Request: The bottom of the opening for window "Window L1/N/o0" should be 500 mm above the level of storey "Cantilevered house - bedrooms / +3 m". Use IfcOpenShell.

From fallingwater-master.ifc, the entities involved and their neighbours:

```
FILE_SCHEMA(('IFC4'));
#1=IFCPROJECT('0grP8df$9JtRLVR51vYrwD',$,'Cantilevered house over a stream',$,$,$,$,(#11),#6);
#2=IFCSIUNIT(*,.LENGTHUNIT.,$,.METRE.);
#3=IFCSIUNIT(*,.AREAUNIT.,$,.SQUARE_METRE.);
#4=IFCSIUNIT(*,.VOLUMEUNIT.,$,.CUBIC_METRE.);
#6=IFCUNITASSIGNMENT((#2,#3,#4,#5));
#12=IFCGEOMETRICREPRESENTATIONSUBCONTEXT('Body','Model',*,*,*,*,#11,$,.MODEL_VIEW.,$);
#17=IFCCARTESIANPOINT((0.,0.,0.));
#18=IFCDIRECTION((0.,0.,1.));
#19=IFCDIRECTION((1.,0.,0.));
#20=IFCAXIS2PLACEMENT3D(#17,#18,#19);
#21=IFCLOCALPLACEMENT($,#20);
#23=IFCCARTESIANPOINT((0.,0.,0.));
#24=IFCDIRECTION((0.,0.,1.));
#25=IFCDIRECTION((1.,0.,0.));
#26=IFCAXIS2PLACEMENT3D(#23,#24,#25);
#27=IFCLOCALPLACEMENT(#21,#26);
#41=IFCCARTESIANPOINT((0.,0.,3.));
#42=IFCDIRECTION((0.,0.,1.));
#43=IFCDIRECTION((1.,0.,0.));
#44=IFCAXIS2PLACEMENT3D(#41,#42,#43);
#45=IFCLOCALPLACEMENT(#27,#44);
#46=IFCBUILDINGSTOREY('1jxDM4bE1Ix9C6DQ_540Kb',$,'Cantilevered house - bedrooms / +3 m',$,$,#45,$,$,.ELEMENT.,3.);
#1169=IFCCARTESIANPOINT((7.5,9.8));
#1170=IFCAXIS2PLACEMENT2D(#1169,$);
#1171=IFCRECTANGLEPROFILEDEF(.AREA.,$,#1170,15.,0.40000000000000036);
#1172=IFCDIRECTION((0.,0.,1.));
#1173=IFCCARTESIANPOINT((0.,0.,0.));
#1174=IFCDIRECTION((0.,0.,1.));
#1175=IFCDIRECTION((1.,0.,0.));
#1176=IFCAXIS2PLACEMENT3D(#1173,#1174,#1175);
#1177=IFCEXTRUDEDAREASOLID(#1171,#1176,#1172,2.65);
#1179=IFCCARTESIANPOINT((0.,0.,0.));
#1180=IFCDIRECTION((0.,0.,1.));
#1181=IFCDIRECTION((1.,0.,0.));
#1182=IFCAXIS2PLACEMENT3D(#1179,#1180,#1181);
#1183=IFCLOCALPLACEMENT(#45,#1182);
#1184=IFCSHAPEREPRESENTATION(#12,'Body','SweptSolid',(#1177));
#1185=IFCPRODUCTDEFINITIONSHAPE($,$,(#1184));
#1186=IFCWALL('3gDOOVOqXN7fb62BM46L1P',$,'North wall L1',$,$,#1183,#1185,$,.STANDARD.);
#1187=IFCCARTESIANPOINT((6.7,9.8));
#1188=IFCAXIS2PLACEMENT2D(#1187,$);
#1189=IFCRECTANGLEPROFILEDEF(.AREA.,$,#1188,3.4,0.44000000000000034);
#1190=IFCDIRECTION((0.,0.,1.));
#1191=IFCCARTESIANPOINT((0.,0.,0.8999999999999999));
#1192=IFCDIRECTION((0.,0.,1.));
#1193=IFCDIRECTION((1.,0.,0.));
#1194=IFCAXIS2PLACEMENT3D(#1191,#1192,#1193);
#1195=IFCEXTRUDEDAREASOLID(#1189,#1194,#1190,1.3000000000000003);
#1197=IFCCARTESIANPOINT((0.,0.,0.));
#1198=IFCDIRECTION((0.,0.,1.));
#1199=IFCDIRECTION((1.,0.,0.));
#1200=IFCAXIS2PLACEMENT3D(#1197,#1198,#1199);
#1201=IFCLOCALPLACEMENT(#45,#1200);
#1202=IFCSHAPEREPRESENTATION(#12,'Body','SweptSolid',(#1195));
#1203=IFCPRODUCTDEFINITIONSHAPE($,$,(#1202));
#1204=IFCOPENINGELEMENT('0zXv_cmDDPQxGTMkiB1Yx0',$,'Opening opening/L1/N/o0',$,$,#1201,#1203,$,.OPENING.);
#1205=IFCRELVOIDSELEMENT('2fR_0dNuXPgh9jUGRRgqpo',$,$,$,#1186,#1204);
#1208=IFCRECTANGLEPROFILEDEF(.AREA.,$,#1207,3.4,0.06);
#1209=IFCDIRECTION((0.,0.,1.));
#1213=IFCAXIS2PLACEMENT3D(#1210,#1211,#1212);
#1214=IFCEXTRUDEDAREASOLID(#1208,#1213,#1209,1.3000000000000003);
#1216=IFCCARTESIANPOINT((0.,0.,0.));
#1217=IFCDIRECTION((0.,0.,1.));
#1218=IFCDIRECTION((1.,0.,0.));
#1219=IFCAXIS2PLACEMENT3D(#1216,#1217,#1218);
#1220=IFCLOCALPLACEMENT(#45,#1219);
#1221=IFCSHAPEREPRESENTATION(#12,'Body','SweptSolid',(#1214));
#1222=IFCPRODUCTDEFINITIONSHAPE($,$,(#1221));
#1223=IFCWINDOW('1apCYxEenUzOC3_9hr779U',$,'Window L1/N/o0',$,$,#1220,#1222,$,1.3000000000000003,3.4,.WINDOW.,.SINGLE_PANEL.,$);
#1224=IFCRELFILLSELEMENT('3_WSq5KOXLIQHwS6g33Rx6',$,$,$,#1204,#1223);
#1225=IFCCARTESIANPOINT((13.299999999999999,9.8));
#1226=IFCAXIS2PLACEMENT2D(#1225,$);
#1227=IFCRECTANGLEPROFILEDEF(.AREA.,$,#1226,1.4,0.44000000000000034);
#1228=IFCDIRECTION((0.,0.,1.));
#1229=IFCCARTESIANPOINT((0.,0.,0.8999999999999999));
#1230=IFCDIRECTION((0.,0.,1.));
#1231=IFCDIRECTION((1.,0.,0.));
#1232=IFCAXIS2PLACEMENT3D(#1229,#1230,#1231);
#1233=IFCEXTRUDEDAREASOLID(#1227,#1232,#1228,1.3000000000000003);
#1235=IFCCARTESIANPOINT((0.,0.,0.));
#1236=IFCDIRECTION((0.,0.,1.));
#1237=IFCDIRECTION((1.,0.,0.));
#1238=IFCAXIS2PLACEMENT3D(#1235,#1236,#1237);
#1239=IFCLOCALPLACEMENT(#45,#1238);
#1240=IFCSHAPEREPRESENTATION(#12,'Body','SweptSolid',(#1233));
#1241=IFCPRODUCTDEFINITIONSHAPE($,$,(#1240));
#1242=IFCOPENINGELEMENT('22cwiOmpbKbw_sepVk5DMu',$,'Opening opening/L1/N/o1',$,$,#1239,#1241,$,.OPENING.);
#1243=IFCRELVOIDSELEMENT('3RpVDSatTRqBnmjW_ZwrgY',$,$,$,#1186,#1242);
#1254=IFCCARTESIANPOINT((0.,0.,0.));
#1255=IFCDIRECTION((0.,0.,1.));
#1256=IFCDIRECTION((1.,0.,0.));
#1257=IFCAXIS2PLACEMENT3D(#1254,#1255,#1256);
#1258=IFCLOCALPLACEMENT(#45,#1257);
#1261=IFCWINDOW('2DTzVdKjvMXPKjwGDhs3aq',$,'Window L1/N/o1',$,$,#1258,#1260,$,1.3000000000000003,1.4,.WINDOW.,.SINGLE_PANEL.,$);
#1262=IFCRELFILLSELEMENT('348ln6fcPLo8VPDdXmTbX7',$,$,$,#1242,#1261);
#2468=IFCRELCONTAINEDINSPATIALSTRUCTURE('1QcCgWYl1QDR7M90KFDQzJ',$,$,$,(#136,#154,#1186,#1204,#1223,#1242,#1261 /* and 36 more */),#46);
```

```python
import numpy as np
import ifcopenshell
import ifcopenshell.api.geometry
import ifcopenshell.geom
import ifcopenshell.util.element
import ifcopenshell.util.placement
import ifcopenshell.util.shape
import ifcopenshell.util.unit

model = ifcopenshell.open("fallingwater-master.ifc")
unit_scale = ifcopenshell.util.unit.calculate_unit_scale(model)

window = model.by_guid("1apCYxEenUzOC3_9hr779U")
opening = window.FillsVoids[0].RelatingOpeningElement
storey = ifcopenshell.util.element.get_container(window, ifc_class="IfcBuildingStorey")
level = ifcopenshell.util.placement.get_local_placement(storey.ObjectPlacement)[2, 3]

# The opening's origin need not be at the sill, so measure its lowest point.
shape = ifcopenshell.geom.create_shape(ifcopenshell.geom.settings(), opening)
bottom = ifcopenshell.util.shape.get_shape_bottom_elevation(shape, shape.geometry) / unit_scale
dz = level + 0.5 - bottom

shift = np.array([0.0, 0.0, dz])
# The window is not placed relative to its opening, so move both.
for product in (opening, window):
    matrix = ifcopenshell.util.placement.get_local_placement(product.ObjectPlacement)
    matrix[:3, 3] += shift
    ifcopenshell.api.geometry.edit_object_placement(model, product=product, matrix=matrix, is_si=False)

print(f"moved by {dz * unit_scale:+.3f} m")

model.write("fallingwater-master_v2.ifc")
```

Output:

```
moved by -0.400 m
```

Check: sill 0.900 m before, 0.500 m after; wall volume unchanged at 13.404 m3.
